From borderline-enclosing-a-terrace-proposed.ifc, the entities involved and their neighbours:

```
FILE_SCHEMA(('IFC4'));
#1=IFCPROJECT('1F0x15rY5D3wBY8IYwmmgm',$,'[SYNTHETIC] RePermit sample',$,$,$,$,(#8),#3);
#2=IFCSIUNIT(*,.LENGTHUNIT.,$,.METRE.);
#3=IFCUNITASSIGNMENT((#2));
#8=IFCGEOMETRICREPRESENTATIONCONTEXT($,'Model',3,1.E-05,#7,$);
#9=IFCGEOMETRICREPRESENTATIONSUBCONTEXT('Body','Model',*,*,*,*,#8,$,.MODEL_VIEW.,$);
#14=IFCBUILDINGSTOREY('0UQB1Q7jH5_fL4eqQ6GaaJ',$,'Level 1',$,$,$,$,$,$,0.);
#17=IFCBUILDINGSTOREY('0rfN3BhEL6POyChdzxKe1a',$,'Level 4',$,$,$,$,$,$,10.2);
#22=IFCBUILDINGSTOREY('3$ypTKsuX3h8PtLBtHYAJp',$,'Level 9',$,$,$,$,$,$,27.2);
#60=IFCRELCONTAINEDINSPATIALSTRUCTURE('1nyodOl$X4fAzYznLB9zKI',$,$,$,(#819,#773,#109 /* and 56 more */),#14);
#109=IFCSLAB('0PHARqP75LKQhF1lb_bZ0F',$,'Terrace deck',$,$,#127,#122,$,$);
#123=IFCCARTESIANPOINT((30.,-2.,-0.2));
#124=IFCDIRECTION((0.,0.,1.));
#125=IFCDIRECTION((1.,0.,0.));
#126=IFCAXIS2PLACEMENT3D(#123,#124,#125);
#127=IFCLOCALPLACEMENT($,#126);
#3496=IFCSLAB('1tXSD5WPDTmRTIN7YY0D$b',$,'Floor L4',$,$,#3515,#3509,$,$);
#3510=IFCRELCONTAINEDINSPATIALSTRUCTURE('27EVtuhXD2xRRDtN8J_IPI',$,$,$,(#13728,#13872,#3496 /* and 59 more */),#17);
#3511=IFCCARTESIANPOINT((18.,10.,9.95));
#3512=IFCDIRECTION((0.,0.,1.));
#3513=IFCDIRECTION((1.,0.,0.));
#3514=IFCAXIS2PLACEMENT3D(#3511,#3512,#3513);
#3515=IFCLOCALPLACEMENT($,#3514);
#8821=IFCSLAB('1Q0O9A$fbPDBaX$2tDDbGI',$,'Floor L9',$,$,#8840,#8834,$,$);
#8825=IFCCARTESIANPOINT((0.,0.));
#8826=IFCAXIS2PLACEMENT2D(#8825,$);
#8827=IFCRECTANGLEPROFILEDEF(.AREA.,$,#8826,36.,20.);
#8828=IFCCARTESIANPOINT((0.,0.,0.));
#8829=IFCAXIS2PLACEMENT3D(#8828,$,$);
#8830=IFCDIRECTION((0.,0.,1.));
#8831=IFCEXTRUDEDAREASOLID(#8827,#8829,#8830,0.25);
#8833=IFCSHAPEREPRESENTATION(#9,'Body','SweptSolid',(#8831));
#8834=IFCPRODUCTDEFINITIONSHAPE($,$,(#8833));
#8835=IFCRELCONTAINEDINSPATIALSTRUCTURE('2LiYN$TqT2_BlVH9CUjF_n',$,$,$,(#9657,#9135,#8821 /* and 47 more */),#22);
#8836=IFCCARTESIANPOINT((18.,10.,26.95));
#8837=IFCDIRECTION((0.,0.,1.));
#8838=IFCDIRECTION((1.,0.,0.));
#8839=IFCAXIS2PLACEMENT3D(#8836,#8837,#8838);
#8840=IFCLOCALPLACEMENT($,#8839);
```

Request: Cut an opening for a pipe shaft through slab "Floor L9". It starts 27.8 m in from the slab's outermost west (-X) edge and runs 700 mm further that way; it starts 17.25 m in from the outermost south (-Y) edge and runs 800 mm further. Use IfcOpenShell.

```python
import numpy as np
import ifcopenshell
import ifcopenshell.api.feature
import ifcopenshell.api.geometry
import ifcopenshell.api.root
import ifcopenshell.geom
import ifcopenshell.util.placement
import ifcopenshell.util.representation
import ifcopenshell.util.shape
import ifcopenshell.util.unit

model = ifcopenshell.open("borderline-enclosing-a-terrace-proposed.ifc")
unit_scale = ifcopenshell.util.unit.calculate_unit_scale(model)
settings = ifcopenshell.geom.settings()


def volume(element):
    """Net volume in cubic metres, openings subtracted."""
    shape = ifcopenshell.geom.create_shape(settings, element)
    return ifcopenshell.util.shape.get_volume(shape.geometry)


slab = model.by_guid("1Q0O9A$fbPDBaX$2tDDbGI")
before = volume(slab)

# Extent in the slab's own axes, in metres. The edges named are its -X and -Y sides.
slab_shape = ifcopenshell.geom.create_shape(settings, slab)
vertices = ifcopenshell.util.shape.get_vertices(slab_shape.geometry)
x_min, y_min, bottom = vertices.min(axis=0)
top = vertices[:, 2].max()

opening = ifcopenshell.api.root.create_entity(model, ifc_class="IfcOpeningElement", name="Pipe shaft opening", predefined_type="OPENING")
context = ifcopenshell.util.representation.get_context(model, "Model", "Body", "MODEL_VIEW")
width, depth = 0.7, 0.8
outline = [(0.0, 0.0), (width, 0.0), (width, depth), (0.0, depth), (0.0, 0.0)]
# Overshoot both faces by 50 mm so the cut is clean.
shape = ifcopenshell.api.geometry.add_slab_representation(
    model, context=context, depth=top - bottom + 0.1, polyline=outline
)
ifcopenshell.api.geometry.assign_representation(model, product=opening, representation=shape)

matrix = ifcopenshell.util.placement.get_local_placement(slab.ObjectPlacement)
matrix[:, 3] = matrix @ np.append(np.array([x_min + 27.8, y_min + 17.25, bottom - 0.05]) / unit_scale, 1.0)
ifcopenshell.api.geometry.edit_object_placement(model, product=opening, matrix=matrix, is_si=False)
ifcopenshell.api.feature.add_feature(model, feature=opening, element=slab)

after = volume(slab)

print(f"slab volume {before:.3f} -> {after:.3f} m3")

model.write("borderline-enclosing-a-terrace-proposed_rev.ifc")
```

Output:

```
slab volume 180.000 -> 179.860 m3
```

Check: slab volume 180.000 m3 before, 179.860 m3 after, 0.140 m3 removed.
